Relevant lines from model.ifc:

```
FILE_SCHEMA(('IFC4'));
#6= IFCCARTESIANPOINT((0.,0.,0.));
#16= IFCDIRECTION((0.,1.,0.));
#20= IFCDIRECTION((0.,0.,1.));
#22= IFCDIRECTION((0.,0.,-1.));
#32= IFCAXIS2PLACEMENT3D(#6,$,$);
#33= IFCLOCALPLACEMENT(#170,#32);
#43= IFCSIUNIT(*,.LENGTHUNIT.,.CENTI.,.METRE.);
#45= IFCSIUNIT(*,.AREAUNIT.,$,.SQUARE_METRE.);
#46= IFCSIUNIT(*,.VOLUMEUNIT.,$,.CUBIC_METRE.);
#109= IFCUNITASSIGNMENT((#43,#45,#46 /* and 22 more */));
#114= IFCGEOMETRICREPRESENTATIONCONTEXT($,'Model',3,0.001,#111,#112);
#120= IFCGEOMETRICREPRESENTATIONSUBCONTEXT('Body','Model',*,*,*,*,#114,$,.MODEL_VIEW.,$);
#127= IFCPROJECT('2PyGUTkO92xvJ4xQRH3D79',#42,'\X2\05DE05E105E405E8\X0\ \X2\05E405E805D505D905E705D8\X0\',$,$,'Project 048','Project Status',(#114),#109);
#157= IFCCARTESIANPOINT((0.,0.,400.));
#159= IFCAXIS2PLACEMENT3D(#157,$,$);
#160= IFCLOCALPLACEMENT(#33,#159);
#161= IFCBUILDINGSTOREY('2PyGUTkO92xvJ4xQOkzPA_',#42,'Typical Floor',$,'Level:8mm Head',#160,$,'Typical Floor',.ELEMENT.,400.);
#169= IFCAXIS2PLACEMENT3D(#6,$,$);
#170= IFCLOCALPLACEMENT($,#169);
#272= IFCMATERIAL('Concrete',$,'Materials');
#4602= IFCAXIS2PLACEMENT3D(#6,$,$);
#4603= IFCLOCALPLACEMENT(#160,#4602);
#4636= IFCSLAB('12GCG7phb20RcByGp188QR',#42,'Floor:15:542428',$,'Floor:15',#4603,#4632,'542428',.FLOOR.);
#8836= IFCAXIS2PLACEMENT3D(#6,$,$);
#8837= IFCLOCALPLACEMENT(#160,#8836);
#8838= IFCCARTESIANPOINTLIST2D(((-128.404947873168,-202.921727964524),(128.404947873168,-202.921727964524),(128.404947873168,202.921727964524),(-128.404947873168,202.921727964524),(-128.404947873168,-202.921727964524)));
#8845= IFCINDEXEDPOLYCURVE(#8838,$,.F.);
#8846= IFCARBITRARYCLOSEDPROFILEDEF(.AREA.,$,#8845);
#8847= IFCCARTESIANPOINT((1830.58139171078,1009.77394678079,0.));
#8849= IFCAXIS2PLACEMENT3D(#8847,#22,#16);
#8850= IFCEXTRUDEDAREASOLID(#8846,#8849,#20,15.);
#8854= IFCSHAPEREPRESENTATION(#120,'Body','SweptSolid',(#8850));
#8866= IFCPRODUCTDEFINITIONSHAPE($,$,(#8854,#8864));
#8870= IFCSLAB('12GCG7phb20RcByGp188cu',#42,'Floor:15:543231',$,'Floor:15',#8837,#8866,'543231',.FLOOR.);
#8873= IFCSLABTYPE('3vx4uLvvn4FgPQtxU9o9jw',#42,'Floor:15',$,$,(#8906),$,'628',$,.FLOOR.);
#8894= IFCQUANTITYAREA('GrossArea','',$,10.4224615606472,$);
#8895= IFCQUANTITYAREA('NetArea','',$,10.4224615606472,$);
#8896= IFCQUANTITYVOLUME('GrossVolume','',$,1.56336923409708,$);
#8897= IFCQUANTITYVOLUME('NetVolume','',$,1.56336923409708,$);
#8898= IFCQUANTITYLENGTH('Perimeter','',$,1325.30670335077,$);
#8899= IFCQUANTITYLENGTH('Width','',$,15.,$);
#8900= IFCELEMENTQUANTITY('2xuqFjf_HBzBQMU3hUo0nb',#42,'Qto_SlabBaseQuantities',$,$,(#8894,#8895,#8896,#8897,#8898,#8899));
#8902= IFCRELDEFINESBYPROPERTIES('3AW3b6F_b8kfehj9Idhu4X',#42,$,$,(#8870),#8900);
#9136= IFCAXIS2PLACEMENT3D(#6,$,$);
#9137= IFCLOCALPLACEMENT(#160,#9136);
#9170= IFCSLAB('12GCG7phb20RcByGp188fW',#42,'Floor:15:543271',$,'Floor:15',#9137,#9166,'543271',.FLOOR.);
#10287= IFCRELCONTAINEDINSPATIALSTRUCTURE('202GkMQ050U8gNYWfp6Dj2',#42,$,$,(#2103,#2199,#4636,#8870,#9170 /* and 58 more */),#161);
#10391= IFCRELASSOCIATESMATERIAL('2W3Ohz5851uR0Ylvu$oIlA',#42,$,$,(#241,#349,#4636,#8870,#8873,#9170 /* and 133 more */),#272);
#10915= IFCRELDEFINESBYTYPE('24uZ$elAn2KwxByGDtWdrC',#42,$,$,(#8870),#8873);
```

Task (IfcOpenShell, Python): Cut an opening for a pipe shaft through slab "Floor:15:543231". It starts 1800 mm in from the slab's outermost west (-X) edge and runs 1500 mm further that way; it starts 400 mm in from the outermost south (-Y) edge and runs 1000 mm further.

```python
import numpy as np
import ifcopenshell
import ifcopenshell.api.feature
import ifcopenshell.api.geometry
import ifcopenshell.api.pset
import ifcopenshell.api.root
import ifcopenshell.geom
import ifcopenshell.util.element
import ifcopenshell.util.placement
import ifcopenshell.util.representation
import ifcopenshell.util.shape
import ifcopenshell.util.unit

model = ifcopenshell.open("model.ifc")
unit_scale = ifcopenshell.util.unit.calculate_unit_scale(model)
area_scale = ifcopenshell.util.unit.calculate_unit_scale(model, "AREAUNIT")
volume_scale = ifcopenshell.util.unit.calculate_unit_scale(model, "VOLUMEUNIT")
settings = ifcopenshell.geom.settings()


def volume(element):
    """Net volume in cubic metres, openings subtracted."""
    shape = ifcopenshell.geom.create_shape(settings, element)
    return ifcopenshell.util.shape.get_volume(shape.geometry)


slab = model.by_guid("12GCG7phb20RcByGp188cu")
before = volume(slab)

# Extent in the slab's own axes, in metres. The edges named are its -X and -Y sides.
slab_shape = ifcopenshell.geom.create_shape(settings, slab)
vertices = ifcopenshell.util.shape.get_vertices(slab_shape.geometry)
x_min, y_min, bottom = vertices.min(axis=0)
top = vertices[:, 2].max()

opening = ifcopenshell.api.root.create_entity(model, ifc_class="IfcOpeningElement", name="Pipe shaft opening", predefined_type="OPENING")
context = ifcopenshell.util.representation.get_context(model, "Model", "Body", "MODEL_VIEW")
width, depth = 1.5, 1
outline = [(0.0, 0.0), (width, 0.0), (width, depth), (0.0, depth), (0.0, 0.0)]
# Overshoot both faces by 50 mm so the cut is clean.
shape = ifcopenshell.api.geometry.add_slab_representation(
    model, context=context, depth=top - bottom + 0.1, polyline=outline
)
ifcopenshell.api.geometry.assign_representation(model, product=opening, representation=shape)

matrix = ifcopenshell.util.placement.get_local_placement(slab.ObjectPlacement)
matrix[:, 3] = matrix @ np.append(np.array([x_min + 1.8, y_min + 0.4, bottom - 0.05]) / unit_scale, 1.0)
ifcopenshell.api.geometry.edit_object_placement(model, product=opening, matrix=matrix, is_si=False)
ifcopenshell.api.feature.add_feature(model, feature=opening, element=slab)

after = volume(slab)

# Update the slab's stored quantities.
qto = model.by_id(ifcopenshell.util.element.get_pset(slab, "Qto_SlabBaseQuantities", should_inherit=False)["id"])
ifcopenshell.api.pset.edit_qto(model, qto=qto, properties={
    "NetArea": after / (top - bottom) / area_scale,
    "NetVolume": after / volume_scale,
})

print(f"slab volume {before:.3f} -> {after:.3f} m3")

model.write("model_v2.ifc")
```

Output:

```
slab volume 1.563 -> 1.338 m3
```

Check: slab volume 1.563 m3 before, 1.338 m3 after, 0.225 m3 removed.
